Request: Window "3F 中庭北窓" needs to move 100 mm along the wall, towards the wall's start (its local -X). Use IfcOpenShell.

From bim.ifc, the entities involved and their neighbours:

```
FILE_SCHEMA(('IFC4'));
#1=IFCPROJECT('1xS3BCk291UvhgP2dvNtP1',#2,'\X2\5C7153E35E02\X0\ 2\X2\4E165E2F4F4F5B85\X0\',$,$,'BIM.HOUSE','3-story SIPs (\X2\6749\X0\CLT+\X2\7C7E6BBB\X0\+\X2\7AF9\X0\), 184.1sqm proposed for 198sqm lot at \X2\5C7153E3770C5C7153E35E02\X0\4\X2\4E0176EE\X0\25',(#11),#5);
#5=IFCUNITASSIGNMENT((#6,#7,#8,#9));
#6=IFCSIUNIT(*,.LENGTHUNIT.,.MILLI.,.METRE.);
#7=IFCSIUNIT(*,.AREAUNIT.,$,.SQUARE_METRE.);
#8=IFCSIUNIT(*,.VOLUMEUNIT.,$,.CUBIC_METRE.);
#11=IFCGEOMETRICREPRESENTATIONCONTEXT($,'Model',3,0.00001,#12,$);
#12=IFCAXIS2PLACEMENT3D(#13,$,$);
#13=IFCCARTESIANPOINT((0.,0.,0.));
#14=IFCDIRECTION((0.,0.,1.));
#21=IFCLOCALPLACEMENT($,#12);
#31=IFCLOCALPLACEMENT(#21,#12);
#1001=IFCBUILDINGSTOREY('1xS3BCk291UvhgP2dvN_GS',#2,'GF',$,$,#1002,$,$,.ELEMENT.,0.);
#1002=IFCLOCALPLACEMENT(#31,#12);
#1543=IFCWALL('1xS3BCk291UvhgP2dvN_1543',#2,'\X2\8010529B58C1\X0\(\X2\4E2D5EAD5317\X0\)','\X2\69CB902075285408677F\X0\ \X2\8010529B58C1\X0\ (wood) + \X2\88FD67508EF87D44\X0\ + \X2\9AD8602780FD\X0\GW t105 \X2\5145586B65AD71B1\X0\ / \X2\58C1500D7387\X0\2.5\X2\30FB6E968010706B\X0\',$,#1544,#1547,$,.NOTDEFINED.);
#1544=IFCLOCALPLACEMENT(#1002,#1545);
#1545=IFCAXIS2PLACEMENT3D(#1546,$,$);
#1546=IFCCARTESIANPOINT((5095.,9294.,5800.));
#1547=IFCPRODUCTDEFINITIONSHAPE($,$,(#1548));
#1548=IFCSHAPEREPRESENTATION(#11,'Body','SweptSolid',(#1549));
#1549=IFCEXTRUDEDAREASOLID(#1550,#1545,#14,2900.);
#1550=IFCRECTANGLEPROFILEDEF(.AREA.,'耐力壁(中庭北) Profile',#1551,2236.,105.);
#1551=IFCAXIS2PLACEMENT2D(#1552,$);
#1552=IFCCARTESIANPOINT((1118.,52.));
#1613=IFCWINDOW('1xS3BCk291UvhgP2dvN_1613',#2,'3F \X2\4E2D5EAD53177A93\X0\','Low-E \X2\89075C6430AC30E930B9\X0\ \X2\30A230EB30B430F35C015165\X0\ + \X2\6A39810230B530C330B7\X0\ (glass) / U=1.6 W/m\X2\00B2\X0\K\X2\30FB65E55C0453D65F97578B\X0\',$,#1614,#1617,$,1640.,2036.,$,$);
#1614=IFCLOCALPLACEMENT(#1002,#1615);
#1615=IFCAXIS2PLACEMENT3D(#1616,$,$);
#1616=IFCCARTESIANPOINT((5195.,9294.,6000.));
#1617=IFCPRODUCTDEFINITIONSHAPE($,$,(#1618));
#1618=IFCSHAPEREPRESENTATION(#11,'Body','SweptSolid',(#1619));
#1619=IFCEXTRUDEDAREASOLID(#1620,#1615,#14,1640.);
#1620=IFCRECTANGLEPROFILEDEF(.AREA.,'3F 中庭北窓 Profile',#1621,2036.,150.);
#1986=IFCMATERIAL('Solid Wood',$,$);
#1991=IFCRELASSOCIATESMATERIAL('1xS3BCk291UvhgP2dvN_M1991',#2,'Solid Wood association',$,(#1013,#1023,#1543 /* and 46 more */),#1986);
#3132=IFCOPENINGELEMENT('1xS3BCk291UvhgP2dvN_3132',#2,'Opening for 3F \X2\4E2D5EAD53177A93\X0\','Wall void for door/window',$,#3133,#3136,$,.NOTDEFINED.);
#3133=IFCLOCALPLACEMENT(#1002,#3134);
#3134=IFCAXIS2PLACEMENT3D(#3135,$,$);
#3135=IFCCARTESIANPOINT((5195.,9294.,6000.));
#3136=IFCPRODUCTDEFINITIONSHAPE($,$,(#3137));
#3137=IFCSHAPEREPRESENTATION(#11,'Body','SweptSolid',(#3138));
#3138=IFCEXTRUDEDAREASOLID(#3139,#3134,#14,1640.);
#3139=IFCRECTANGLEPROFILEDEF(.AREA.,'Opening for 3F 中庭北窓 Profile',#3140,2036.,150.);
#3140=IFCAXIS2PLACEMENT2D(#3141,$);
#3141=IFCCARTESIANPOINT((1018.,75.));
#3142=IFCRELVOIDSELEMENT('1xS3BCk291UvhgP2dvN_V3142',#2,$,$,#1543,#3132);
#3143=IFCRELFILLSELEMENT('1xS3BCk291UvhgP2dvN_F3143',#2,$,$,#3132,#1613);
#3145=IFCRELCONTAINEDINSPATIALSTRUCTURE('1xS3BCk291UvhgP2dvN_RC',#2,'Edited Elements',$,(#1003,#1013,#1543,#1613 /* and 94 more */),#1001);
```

```python
import ifcopenshell
import ifcopenshell.api.geometry
import ifcopenshell.util.placement
import ifcopenshell.util.unit

model = ifcopenshell.open("bim.ifc")
unit_scale = ifcopenshell.util.unit.calculate_unit_scale(model)

window = model.by_guid("1xS3BCk291UvhgP2dvN_1613")
opening = window.FillsVoids[0].RelatingOpeningElement
wall = opening.VoidsElements[0].RelatingBuildingElement

wall_matrix = ifcopenshell.util.placement.get_local_placement(wall.ObjectPlacement)
shift = wall_matrix[:3, 0] * -0.1 / unit_scale
before = ifcopenshell.util.placement.get_local_placement(window.ObjectPlacement)[:3, 3].copy()

# The window is not placed relative to its opening, so move both.
for product in (opening, window):
    matrix = ifcopenshell.util.placement.get_local_placement(product.ObjectPlacement)
    matrix[:3, 3] += shift
    ifcopenshell.api.geometry.edit_object_placement(model, product=product, matrix=matrix, is_si=False)

after = ifcopenshell.util.placement.get_local_placement(window.ObjectPlacement)[:3, 3]
print("window moved by", (after - before).round(3) + 0.0)

model.write("bim_v2.ifc")
```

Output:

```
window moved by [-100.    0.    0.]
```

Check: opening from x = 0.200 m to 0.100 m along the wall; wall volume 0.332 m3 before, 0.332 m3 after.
